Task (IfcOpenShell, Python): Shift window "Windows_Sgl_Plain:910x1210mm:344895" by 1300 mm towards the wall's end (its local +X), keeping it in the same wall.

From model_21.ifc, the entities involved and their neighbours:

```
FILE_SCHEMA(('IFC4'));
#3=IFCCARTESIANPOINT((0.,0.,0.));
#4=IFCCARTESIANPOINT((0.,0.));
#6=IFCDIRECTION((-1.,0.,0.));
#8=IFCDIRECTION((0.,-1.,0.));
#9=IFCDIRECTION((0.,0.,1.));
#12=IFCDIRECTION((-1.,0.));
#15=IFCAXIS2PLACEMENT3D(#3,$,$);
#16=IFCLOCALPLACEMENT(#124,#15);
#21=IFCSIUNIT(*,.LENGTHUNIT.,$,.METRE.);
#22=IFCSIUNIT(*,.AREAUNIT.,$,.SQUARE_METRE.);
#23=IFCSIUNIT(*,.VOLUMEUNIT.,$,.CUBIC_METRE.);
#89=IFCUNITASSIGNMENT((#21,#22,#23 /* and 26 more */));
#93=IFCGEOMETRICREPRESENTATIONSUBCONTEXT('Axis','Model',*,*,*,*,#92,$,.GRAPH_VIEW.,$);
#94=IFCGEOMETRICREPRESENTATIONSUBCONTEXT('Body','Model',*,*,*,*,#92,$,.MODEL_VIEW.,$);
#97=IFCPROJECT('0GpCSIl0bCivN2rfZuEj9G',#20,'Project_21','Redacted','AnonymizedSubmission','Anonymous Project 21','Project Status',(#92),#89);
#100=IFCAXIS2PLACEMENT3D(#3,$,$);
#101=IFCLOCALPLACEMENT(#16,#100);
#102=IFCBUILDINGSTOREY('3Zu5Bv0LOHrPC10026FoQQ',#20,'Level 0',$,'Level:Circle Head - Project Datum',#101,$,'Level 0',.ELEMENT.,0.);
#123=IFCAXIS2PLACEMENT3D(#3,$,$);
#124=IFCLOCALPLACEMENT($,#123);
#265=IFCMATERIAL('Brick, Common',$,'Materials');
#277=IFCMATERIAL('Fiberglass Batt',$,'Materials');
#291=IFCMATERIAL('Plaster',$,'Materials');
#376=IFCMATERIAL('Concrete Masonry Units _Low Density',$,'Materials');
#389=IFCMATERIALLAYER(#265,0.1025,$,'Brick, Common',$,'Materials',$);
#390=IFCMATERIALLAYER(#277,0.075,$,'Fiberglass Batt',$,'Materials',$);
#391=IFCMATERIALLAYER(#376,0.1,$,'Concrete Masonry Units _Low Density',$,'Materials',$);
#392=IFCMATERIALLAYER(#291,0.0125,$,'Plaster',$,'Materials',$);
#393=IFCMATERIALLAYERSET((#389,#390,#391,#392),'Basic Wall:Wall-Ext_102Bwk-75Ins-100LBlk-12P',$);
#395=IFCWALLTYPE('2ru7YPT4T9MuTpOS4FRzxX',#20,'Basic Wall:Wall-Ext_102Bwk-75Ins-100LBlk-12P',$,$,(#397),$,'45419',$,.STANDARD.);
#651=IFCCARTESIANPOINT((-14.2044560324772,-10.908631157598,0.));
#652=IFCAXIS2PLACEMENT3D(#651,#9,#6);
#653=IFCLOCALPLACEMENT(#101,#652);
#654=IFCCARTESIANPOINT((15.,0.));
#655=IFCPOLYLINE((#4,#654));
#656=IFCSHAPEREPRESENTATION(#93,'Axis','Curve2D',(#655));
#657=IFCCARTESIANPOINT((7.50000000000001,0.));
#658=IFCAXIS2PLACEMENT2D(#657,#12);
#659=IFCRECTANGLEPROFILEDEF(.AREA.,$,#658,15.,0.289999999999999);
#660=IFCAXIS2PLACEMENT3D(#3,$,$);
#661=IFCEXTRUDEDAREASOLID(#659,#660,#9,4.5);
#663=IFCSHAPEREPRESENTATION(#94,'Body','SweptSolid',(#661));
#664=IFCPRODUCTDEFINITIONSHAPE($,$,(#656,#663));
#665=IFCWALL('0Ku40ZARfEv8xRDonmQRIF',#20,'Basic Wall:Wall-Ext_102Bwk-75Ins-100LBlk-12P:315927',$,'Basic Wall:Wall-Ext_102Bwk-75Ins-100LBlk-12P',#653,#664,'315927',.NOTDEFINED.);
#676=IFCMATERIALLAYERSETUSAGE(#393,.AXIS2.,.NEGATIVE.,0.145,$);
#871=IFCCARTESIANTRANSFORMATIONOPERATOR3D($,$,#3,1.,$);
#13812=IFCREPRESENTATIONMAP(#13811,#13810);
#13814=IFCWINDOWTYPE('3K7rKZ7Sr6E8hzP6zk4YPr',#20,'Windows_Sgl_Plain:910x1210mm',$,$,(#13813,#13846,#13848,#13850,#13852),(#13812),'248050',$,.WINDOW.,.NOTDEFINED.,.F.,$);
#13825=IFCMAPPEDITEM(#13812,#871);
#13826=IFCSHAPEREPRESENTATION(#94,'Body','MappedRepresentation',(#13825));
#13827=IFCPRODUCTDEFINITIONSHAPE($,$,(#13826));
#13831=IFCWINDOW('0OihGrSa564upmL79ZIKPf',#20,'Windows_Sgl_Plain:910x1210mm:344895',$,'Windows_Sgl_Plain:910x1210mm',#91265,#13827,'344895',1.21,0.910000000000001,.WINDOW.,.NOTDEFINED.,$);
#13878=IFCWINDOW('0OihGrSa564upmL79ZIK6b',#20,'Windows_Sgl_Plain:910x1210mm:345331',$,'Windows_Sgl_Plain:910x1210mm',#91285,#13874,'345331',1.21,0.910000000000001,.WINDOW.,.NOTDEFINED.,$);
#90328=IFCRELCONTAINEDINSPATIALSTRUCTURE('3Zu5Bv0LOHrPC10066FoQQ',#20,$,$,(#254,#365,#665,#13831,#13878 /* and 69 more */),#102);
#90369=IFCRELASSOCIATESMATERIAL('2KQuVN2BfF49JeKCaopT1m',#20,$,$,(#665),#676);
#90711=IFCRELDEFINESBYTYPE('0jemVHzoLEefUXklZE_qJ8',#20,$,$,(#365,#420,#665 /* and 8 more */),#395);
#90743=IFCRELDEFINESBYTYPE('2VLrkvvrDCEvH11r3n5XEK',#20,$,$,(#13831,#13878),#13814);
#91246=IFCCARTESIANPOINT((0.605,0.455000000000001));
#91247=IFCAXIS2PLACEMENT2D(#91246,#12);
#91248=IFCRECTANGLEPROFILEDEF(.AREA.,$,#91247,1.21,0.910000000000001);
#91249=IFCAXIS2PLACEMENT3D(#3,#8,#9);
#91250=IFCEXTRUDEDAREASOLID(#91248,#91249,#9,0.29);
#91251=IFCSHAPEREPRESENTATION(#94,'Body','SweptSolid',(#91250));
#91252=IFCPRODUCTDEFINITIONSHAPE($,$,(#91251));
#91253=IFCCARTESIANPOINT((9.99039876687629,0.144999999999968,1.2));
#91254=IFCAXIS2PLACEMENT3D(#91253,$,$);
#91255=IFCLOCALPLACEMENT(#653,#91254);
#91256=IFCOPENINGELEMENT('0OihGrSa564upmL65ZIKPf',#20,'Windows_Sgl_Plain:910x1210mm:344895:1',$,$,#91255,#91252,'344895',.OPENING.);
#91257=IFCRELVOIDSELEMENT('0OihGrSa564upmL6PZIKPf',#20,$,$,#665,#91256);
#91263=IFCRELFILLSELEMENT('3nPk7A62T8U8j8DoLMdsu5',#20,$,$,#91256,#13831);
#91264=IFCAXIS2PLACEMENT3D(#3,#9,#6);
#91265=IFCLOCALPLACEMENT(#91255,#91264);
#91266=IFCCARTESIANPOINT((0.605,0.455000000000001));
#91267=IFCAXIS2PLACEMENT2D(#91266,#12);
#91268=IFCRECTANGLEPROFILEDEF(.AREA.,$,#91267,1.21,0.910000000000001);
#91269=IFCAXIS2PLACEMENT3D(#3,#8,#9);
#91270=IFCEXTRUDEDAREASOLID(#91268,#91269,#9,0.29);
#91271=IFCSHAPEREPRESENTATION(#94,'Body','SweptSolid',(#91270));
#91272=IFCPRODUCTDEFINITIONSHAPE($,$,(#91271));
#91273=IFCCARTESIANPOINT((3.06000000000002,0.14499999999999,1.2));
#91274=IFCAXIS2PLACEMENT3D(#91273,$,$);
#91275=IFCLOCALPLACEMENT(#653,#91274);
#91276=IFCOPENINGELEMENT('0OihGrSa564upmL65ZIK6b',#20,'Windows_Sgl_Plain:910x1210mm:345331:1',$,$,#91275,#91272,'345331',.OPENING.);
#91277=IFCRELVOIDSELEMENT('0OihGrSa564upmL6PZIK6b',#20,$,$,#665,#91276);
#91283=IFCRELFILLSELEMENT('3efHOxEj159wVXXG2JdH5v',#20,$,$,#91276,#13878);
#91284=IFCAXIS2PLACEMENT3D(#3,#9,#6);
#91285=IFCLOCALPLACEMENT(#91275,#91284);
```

```python
import ifcopenshell
import ifcopenshell.api.geometry
import ifcopenshell.util.placement

model = ifcopenshell.open("model_21.ifc")

window = model.by_guid("0OihGrSa564upmL79ZIKPf")
opening = window.FillsVoids[0].RelatingOpeningElement
wall = opening.VoidsElements[0].RelatingBuildingElement

wall_matrix = ifcopenshell.util.placement.get_local_placement(wall.ObjectPlacement)
shift = wall_matrix[:3, 0] * 1.3
before = ifcopenshell.util.placement.get_local_placement(window.ObjectPlacement)[:3, 3].copy()

# The window is placed relative to its opening, so it follows when the opening moves.
matrix = ifcopenshell.util.placement.get_local_placement(opening.ObjectPlacement)
matrix[:3, 3] += shift
ifcopenshell.api.geometry.edit_object_placement(
    model, product=opening, matrix=matrix, is_si=False, should_transform_children=True
)

after = ifcopenshell.util.placement.get_local_placement(window.ObjectPlacement)[:3, 3]
print("window moved by", (after - before).round(3) + 0.0)

model.write("model_21-out.ifc")
```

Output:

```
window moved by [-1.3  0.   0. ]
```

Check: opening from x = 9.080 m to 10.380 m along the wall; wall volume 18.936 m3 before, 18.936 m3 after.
